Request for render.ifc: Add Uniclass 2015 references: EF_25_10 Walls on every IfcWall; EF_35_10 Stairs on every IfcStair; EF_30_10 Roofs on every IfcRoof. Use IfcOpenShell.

First a look at what the model holds.

```python
import ifcopenshell

model = ifcopenshell.open("render.ifc")
print(model.schema)
print("classifications:", [c.Name for c in model.by_type("IfcClassification")])
for ifc_class in ("IfcDoor", "IfcRoof", "IfcStair", "IfcWall", "IfcWindow"):
    print(ifc_class, len(model.by_type(ifc_class)))
```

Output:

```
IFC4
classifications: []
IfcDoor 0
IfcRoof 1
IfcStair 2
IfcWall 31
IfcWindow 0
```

```python
import ifcopenshell
import ifcopenshell.api.classification

model = ifcopenshell.open("render.ifc")

system = ifcopenshell.api.classification.add_classification(model, classification="Uniclass 2015")

codes = {
    "IfcWall": ("EF_25_10", "Walls"),
    "IfcStair": ("EF_35_10", "Stairs"),
    "IfcRoof": ("EF_30_10", "Roofs"),
}
for ifc_class, (code, name) in codes.items():
    products = model.by_type(ifc_class)
    ifcopenshell.api.classification.add_reference(
        model, products=products, classification=system, identification=code, name=name
    )
    print(code, len(products))

model.write("render_rev.ifc")
```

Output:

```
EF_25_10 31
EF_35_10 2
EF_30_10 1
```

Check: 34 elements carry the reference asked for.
